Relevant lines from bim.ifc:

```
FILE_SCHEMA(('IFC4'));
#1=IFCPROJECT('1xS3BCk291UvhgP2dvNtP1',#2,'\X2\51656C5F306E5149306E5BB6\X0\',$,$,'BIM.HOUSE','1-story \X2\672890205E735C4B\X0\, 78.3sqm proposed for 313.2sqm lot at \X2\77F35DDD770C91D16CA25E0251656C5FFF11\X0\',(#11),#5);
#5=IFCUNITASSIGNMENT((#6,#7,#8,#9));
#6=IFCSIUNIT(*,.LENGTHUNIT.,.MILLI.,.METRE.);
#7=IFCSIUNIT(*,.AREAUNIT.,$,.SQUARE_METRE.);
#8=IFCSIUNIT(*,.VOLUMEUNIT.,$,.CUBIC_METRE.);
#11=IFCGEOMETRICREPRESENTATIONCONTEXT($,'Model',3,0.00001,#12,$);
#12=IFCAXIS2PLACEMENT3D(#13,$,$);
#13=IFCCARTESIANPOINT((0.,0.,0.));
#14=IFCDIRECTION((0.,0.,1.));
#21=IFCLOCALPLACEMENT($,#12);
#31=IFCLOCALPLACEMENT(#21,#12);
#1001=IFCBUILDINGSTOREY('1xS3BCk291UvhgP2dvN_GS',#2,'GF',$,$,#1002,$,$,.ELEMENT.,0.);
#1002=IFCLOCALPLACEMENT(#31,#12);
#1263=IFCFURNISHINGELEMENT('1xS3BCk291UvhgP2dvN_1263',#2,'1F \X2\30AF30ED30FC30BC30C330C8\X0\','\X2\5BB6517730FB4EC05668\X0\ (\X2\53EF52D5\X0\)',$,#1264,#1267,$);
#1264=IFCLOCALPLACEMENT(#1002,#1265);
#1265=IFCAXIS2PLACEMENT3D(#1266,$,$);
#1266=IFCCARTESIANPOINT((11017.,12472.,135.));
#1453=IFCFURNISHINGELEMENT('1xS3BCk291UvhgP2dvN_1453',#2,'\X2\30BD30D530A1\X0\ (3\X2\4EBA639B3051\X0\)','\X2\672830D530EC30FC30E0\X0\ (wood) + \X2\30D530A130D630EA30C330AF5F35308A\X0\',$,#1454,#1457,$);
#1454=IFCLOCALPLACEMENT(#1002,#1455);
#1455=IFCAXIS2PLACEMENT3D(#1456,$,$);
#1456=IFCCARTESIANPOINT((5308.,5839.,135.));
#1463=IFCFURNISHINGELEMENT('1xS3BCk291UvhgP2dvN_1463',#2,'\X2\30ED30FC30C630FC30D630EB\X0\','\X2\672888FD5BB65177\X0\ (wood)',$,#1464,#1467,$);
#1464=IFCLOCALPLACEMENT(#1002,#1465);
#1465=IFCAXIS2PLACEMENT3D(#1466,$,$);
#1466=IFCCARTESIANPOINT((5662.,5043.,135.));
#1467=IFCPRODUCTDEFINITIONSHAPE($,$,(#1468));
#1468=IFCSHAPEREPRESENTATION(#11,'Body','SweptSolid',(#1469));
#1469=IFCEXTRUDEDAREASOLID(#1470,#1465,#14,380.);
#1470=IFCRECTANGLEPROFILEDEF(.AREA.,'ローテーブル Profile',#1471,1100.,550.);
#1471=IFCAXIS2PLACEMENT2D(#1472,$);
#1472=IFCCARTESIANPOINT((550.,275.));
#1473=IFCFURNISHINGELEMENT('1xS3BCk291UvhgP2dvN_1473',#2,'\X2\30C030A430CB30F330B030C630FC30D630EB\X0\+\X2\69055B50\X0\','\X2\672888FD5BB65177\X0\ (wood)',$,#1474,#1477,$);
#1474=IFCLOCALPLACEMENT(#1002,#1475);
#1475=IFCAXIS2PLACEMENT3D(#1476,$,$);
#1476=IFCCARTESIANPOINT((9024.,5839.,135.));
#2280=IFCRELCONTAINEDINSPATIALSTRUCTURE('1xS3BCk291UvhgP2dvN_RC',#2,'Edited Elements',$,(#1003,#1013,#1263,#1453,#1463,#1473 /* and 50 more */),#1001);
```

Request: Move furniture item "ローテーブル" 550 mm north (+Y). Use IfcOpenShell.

```python
import ifcopenshell
import ifcopenshell.api.geometry
import ifcopenshell.util.placement
import ifcopenshell.util.unit

model = ifcopenshell.open("bim.ifc")
unit_scale = ifcopenshell.util.unit.calculate_unit_scale(model)

item = model.by_id(1463)
matrix = ifcopenshell.util.placement.get_local_placement(item.ObjectPlacement)
matrix[1, 3] += 0.55 / unit_scale
ifcopenshell.api.geometry.edit_object_placement(model, product=item, matrix=matrix, is_si=False)

print(ifcopenshell.util.placement.get_local_placement(item.ObjectPlacement).round(3) + 0.0)

model.write("bim_rev.ifc")
```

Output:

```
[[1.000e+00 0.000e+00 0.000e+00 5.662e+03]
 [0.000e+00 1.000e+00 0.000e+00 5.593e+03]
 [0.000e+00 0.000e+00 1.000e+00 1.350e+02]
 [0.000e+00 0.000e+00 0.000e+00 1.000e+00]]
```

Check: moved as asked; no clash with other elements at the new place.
